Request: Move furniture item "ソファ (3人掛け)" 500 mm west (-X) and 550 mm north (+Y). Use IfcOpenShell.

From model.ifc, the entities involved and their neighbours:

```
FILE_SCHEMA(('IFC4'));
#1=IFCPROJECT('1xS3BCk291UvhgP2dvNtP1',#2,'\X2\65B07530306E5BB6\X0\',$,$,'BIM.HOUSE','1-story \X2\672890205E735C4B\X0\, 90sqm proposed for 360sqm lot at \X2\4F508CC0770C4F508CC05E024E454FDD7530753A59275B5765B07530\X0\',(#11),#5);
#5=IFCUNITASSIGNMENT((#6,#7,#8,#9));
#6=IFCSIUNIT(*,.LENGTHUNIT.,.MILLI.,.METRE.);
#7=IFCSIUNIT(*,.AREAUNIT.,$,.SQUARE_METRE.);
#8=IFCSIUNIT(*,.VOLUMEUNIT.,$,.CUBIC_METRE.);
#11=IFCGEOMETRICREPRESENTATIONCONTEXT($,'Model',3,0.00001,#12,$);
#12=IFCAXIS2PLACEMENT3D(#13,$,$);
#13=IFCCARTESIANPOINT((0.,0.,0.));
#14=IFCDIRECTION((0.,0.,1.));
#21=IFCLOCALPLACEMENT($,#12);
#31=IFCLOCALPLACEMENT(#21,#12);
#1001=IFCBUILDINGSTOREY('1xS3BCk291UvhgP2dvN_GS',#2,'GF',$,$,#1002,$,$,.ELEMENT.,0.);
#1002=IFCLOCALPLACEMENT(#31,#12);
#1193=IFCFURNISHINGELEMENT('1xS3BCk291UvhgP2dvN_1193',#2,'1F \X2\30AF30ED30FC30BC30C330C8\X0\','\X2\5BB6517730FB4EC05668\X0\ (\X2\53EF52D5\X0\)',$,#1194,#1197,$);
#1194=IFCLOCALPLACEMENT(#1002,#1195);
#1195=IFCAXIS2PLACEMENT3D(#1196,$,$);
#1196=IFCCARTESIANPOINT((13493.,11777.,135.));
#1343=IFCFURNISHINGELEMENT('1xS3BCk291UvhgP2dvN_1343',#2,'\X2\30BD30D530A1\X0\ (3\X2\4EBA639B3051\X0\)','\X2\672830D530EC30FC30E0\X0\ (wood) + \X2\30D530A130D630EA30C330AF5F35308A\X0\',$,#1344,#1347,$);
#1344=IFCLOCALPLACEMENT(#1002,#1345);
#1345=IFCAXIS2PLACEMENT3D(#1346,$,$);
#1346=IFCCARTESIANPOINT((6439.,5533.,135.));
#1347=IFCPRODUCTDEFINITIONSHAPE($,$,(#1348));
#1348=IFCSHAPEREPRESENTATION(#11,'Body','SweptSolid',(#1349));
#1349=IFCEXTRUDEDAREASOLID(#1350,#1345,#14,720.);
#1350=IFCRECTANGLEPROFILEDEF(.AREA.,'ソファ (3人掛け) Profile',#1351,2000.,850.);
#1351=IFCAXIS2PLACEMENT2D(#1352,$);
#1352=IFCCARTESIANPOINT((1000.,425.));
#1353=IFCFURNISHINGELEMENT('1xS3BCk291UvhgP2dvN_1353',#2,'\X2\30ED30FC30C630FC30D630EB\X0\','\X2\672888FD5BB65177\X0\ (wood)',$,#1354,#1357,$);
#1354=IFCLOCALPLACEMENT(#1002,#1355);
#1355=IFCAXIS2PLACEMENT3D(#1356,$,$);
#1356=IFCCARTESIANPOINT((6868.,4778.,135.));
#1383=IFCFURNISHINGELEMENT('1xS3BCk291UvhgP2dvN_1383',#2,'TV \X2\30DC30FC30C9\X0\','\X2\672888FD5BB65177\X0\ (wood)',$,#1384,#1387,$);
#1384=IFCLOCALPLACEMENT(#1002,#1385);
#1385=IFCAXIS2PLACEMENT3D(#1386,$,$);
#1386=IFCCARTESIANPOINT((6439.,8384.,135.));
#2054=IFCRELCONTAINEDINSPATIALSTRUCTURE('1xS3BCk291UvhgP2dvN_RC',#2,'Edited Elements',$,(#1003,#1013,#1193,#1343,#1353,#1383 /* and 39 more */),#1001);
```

```python
import ifcopenshell
import ifcopenshell.api.geometry
import ifcopenshell.util.placement
import ifcopenshell.util.unit

model = ifcopenshell.open("model.ifc")
unit_scale = ifcopenshell.util.unit.calculate_unit_scale(model)

item = model.by_guid("1xS3BCk291UvhgP2dvN_1343")
matrix = ifcopenshell.util.placement.get_local_placement(item.ObjectPlacement)
matrix[0, 3] -= 0.5 / unit_scale
matrix[1, 3] += 0.55 / unit_scale
ifcopenshell.api.geometry.edit_object_placement(model, product=item, matrix=matrix, is_si=False)

print(ifcopenshell.util.placement.get_local_placement(item.ObjectPlacement).round(3) + 0.0)

model.write("model-out.ifc")
```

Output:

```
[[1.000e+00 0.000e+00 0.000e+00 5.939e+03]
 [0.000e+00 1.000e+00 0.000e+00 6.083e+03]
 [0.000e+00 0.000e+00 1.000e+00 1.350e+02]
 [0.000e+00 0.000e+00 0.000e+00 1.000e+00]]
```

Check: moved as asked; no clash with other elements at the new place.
